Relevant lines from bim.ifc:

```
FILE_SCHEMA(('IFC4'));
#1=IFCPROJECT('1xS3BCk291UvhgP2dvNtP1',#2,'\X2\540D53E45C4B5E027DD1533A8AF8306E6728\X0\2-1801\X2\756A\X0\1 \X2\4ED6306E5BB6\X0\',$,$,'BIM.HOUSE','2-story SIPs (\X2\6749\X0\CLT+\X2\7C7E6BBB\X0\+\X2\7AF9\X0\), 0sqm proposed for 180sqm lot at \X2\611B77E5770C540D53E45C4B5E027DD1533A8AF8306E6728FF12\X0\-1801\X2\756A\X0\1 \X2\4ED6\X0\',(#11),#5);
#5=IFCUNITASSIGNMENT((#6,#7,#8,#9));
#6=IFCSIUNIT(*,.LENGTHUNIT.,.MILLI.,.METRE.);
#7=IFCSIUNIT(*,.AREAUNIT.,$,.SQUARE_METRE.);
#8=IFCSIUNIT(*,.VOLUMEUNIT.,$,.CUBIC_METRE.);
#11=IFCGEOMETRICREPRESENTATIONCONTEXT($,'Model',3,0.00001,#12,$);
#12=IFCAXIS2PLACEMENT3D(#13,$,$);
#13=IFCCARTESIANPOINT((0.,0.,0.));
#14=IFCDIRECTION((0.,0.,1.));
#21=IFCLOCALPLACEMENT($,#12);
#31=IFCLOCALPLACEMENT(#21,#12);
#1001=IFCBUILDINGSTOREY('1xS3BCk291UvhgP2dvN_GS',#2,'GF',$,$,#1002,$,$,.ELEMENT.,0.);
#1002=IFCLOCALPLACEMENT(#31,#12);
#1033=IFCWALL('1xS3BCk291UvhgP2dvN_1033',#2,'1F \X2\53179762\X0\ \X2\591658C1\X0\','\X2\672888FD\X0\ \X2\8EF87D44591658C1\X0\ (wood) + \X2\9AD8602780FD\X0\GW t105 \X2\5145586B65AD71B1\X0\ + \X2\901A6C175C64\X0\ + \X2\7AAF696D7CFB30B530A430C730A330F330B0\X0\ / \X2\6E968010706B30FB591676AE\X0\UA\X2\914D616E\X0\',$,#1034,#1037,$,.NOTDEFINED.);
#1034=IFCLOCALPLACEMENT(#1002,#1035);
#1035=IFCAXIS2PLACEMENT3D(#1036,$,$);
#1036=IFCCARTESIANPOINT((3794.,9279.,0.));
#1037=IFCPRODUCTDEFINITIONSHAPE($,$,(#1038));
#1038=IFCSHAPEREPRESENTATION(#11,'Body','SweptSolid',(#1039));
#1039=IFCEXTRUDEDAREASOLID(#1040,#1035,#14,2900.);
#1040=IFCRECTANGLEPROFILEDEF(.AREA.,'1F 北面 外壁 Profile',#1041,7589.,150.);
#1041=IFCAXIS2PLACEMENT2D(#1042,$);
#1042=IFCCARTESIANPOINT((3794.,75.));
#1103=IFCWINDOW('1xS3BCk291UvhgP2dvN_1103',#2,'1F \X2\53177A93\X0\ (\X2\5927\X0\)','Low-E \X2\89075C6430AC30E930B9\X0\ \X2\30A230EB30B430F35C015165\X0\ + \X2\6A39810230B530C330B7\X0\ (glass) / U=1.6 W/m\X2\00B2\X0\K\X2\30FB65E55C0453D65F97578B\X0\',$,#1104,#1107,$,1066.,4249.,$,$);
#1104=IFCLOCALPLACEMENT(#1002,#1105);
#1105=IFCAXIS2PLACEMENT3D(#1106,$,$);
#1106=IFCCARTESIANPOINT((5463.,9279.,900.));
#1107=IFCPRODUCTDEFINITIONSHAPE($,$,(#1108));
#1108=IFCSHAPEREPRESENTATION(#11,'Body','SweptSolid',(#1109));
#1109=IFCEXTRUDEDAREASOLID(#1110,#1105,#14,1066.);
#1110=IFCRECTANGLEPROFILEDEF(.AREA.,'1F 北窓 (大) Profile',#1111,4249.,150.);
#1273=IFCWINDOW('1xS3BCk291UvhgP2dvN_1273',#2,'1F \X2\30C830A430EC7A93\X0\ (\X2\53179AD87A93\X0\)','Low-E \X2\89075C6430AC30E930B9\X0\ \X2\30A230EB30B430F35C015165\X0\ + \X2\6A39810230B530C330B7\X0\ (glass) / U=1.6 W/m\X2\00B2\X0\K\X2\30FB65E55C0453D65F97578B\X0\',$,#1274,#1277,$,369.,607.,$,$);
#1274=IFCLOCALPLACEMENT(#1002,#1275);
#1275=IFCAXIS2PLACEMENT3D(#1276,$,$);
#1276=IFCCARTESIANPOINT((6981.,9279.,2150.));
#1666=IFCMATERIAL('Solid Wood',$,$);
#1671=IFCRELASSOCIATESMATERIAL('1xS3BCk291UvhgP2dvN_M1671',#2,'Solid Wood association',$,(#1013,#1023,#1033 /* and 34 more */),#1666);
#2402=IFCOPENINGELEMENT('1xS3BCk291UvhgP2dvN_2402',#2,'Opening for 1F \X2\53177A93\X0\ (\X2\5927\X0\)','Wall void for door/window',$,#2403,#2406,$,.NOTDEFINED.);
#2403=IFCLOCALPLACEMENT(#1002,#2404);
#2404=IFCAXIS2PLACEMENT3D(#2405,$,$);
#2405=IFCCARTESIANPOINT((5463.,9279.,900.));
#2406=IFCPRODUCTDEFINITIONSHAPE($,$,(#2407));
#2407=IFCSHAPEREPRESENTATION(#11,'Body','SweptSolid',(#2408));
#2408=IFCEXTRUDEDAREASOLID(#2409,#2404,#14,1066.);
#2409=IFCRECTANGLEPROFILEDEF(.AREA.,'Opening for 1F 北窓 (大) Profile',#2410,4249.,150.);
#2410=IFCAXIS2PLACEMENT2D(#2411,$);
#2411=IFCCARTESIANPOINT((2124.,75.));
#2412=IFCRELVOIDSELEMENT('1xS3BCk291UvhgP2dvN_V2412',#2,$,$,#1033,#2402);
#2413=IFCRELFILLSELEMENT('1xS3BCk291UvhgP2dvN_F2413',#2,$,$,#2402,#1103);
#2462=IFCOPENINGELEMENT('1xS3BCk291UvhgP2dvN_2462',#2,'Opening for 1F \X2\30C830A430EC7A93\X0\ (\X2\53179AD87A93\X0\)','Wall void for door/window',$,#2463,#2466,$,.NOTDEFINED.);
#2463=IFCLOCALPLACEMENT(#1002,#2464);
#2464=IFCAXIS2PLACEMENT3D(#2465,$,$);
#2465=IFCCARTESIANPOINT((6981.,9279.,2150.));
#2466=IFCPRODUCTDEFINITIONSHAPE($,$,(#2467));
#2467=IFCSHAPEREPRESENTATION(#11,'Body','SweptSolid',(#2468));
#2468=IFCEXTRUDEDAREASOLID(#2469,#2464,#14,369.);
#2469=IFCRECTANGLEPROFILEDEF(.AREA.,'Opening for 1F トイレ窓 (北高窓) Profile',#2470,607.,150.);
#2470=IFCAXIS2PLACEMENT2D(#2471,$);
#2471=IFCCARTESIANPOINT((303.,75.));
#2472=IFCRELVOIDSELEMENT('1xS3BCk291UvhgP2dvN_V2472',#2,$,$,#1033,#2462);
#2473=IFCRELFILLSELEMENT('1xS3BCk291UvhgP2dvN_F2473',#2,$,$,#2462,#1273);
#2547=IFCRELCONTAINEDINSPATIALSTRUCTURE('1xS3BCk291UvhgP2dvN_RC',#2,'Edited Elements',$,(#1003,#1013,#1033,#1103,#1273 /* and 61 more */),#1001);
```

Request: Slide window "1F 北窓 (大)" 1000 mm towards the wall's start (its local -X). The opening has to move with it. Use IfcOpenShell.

```python
import ifcopenshell
import ifcopenshell.api.geometry
import ifcopenshell.util.placement
import ifcopenshell.util.unit

model = ifcopenshell.open("bim.ifc")
unit_scale = ifcopenshell.util.unit.calculate_unit_scale(model)

window = model.by_guid("1xS3BCk291UvhgP2dvN_1103")
opening = window.FillsVoids[0].RelatingOpeningElement
wall = opening.VoidsElements[0].RelatingBuildingElement

wall_matrix = ifcopenshell.util.placement.get_local_placement(wall.ObjectPlacement)
shift = wall_matrix[:3, 0] * -1 / unit_scale
before = ifcopenshell.util.placement.get_local_placement(window.ObjectPlacement)[:3, 3].copy()

# The window is not placed relative to its opening, so move both.
for product in (opening, window):
    matrix = ifcopenshell.util.placement.get_local_placement(product.ObjectPlacement)
    matrix[:3, 3] += shift
    ifcopenshell.api.geometry.edit_object_placement(model, product=product, matrix=matrix, is_si=False)

after = ifcopenshell.util.placement.get_local_placement(window.ObjectPlacement)[:3, 3]
print("window moved by", (after - before).round(3) + 0.0)

model.write("bim_rev.ifc")
```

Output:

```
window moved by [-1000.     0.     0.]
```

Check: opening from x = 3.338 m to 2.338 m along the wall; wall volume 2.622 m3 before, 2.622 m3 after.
